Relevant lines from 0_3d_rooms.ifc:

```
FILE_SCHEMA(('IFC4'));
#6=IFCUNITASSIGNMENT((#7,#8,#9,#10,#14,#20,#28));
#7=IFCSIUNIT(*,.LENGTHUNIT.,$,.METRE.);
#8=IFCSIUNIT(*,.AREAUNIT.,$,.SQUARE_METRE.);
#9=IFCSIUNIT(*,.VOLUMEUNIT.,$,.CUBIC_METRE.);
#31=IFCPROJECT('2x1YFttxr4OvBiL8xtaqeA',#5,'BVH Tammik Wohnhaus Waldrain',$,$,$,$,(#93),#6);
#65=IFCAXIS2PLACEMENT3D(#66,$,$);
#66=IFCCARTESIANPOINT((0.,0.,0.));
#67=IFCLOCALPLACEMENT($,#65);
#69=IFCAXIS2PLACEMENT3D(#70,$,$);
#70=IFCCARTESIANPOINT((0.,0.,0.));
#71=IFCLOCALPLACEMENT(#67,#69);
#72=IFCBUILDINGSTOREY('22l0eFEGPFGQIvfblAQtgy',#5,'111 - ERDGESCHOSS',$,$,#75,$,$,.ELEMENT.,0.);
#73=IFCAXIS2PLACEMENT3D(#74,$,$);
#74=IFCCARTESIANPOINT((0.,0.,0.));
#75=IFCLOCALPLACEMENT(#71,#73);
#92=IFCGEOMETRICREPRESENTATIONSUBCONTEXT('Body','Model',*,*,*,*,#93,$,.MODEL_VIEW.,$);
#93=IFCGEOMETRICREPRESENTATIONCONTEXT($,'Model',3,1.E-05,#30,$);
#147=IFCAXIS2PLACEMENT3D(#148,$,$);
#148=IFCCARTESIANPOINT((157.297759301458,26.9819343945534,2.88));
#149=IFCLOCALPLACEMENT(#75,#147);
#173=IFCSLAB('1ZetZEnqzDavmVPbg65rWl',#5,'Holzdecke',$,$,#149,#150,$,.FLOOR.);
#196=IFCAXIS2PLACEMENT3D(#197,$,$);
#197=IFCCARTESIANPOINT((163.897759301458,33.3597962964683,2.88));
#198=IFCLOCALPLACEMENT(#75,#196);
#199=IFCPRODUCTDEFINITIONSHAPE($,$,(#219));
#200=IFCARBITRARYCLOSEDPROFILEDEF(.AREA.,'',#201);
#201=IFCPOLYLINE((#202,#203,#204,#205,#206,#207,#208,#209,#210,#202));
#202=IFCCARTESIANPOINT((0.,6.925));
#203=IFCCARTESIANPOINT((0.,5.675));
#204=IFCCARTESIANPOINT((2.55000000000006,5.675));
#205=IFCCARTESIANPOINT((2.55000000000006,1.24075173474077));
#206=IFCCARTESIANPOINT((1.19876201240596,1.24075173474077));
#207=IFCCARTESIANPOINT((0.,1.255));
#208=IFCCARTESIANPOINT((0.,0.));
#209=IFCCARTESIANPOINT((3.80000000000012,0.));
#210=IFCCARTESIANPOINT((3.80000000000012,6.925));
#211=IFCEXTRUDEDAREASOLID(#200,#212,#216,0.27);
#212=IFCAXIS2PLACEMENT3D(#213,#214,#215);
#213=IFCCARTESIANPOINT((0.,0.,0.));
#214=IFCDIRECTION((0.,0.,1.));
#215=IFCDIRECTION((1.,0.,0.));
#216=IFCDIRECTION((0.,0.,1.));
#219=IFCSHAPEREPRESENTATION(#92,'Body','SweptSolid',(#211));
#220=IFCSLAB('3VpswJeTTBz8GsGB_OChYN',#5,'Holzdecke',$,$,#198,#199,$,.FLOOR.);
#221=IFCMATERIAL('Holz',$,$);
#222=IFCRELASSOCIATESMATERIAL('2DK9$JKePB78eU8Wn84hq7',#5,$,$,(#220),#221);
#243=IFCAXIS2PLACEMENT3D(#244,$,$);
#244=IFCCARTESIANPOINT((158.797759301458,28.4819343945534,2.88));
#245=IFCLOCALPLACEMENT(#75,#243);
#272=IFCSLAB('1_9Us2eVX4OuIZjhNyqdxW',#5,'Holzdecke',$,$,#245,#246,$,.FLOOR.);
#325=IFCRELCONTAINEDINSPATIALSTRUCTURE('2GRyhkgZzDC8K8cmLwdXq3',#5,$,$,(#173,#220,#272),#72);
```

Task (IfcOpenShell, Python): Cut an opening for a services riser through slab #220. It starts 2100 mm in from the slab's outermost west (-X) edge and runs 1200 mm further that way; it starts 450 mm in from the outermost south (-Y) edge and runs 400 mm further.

```python
import numpy as np
import ifcopenshell
import ifcopenshell.api.feature
import ifcopenshell.api.geometry
import ifcopenshell.api.root
import ifcopenshell.geom
import ifcopenshell.util.placement
import ifcopenshell.util.representation
import ifcopenshell.util.shape
import ifcopenshell.util.unit

model = ifcopenshell.open("0_3d_rooms.ifc")
unit_scale = ifcopenshell.util.unit.calculate_unit_scale(model)
settings = ifcopenshell.geom.settings()


def volume(element):
    """Net volume in cubic metres, openings subtracted."""
    shape = ifcopenshell.geom.create_shape(settings, element)
    return ifcopenshell.util.shape.get_volume(shape.geometry)


slab = model.by_guid("3VpswJeTTBz8GsGB_OChYN")
before = volume(slab)

# Extent in the slab's own axes, in metres. The edges named are its -X and -Y sides.
slab_shape = ifcopenshell.geom.create_shape(settings, slab)
vertices = ifcopenshell.util.shape.get_vertices(slab_shape.geometry)
x_min, y_min, bottom = vertices.min(axis=0)
top = vertices[:, 2].max()

opening = ifcopenshell.api.root.create_entity(model, ifc_class="IfcOpeningElement", name="Services riser opening", predefined_type="OPENING")
context = ifcopenshell.util.representation.get_context(model, "Model", "Body", "MODEL_VIEW")
width, depth = 1.2, 0.4
outline = [(0.0, 0.0), (width, 0.0), (width, depth), (0.0, depth), (0.0, 0.0)]
# Overshoot both faces by 50 mm so the cut is clean.
shape = ifcopenshell.api.geometry.add_slab_representation(
    model, context=context, depth=top - bottom + 0.1, polyline=outline
)
ifcopenshell.api.geometry.assign_representation(model, product=opening, representation=shape)

matrix = ifcopenshell.util.placement.get_local_placement(slab.ObjectPlacement)
matrix[:, 3] = matrix @ np.append(np.array([x_min + 2.1, y_min + 0.45, bottom - 0.05]) / unit_scale, 1.0)
ifcopenshell.api.geometry.edit_object_placement(model, product=opening, matrix=matrix, is_si=False)
ifcopenshell.api.feature.add_feature(model, feature=opening, element=slab)

after = volume(slab)

print(f"slab volume {before:.3f} -> {after:.3f} m3")

model.write("0_3d_rooms_updated.ifc")
```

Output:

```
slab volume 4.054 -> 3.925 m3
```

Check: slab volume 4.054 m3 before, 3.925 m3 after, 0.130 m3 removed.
